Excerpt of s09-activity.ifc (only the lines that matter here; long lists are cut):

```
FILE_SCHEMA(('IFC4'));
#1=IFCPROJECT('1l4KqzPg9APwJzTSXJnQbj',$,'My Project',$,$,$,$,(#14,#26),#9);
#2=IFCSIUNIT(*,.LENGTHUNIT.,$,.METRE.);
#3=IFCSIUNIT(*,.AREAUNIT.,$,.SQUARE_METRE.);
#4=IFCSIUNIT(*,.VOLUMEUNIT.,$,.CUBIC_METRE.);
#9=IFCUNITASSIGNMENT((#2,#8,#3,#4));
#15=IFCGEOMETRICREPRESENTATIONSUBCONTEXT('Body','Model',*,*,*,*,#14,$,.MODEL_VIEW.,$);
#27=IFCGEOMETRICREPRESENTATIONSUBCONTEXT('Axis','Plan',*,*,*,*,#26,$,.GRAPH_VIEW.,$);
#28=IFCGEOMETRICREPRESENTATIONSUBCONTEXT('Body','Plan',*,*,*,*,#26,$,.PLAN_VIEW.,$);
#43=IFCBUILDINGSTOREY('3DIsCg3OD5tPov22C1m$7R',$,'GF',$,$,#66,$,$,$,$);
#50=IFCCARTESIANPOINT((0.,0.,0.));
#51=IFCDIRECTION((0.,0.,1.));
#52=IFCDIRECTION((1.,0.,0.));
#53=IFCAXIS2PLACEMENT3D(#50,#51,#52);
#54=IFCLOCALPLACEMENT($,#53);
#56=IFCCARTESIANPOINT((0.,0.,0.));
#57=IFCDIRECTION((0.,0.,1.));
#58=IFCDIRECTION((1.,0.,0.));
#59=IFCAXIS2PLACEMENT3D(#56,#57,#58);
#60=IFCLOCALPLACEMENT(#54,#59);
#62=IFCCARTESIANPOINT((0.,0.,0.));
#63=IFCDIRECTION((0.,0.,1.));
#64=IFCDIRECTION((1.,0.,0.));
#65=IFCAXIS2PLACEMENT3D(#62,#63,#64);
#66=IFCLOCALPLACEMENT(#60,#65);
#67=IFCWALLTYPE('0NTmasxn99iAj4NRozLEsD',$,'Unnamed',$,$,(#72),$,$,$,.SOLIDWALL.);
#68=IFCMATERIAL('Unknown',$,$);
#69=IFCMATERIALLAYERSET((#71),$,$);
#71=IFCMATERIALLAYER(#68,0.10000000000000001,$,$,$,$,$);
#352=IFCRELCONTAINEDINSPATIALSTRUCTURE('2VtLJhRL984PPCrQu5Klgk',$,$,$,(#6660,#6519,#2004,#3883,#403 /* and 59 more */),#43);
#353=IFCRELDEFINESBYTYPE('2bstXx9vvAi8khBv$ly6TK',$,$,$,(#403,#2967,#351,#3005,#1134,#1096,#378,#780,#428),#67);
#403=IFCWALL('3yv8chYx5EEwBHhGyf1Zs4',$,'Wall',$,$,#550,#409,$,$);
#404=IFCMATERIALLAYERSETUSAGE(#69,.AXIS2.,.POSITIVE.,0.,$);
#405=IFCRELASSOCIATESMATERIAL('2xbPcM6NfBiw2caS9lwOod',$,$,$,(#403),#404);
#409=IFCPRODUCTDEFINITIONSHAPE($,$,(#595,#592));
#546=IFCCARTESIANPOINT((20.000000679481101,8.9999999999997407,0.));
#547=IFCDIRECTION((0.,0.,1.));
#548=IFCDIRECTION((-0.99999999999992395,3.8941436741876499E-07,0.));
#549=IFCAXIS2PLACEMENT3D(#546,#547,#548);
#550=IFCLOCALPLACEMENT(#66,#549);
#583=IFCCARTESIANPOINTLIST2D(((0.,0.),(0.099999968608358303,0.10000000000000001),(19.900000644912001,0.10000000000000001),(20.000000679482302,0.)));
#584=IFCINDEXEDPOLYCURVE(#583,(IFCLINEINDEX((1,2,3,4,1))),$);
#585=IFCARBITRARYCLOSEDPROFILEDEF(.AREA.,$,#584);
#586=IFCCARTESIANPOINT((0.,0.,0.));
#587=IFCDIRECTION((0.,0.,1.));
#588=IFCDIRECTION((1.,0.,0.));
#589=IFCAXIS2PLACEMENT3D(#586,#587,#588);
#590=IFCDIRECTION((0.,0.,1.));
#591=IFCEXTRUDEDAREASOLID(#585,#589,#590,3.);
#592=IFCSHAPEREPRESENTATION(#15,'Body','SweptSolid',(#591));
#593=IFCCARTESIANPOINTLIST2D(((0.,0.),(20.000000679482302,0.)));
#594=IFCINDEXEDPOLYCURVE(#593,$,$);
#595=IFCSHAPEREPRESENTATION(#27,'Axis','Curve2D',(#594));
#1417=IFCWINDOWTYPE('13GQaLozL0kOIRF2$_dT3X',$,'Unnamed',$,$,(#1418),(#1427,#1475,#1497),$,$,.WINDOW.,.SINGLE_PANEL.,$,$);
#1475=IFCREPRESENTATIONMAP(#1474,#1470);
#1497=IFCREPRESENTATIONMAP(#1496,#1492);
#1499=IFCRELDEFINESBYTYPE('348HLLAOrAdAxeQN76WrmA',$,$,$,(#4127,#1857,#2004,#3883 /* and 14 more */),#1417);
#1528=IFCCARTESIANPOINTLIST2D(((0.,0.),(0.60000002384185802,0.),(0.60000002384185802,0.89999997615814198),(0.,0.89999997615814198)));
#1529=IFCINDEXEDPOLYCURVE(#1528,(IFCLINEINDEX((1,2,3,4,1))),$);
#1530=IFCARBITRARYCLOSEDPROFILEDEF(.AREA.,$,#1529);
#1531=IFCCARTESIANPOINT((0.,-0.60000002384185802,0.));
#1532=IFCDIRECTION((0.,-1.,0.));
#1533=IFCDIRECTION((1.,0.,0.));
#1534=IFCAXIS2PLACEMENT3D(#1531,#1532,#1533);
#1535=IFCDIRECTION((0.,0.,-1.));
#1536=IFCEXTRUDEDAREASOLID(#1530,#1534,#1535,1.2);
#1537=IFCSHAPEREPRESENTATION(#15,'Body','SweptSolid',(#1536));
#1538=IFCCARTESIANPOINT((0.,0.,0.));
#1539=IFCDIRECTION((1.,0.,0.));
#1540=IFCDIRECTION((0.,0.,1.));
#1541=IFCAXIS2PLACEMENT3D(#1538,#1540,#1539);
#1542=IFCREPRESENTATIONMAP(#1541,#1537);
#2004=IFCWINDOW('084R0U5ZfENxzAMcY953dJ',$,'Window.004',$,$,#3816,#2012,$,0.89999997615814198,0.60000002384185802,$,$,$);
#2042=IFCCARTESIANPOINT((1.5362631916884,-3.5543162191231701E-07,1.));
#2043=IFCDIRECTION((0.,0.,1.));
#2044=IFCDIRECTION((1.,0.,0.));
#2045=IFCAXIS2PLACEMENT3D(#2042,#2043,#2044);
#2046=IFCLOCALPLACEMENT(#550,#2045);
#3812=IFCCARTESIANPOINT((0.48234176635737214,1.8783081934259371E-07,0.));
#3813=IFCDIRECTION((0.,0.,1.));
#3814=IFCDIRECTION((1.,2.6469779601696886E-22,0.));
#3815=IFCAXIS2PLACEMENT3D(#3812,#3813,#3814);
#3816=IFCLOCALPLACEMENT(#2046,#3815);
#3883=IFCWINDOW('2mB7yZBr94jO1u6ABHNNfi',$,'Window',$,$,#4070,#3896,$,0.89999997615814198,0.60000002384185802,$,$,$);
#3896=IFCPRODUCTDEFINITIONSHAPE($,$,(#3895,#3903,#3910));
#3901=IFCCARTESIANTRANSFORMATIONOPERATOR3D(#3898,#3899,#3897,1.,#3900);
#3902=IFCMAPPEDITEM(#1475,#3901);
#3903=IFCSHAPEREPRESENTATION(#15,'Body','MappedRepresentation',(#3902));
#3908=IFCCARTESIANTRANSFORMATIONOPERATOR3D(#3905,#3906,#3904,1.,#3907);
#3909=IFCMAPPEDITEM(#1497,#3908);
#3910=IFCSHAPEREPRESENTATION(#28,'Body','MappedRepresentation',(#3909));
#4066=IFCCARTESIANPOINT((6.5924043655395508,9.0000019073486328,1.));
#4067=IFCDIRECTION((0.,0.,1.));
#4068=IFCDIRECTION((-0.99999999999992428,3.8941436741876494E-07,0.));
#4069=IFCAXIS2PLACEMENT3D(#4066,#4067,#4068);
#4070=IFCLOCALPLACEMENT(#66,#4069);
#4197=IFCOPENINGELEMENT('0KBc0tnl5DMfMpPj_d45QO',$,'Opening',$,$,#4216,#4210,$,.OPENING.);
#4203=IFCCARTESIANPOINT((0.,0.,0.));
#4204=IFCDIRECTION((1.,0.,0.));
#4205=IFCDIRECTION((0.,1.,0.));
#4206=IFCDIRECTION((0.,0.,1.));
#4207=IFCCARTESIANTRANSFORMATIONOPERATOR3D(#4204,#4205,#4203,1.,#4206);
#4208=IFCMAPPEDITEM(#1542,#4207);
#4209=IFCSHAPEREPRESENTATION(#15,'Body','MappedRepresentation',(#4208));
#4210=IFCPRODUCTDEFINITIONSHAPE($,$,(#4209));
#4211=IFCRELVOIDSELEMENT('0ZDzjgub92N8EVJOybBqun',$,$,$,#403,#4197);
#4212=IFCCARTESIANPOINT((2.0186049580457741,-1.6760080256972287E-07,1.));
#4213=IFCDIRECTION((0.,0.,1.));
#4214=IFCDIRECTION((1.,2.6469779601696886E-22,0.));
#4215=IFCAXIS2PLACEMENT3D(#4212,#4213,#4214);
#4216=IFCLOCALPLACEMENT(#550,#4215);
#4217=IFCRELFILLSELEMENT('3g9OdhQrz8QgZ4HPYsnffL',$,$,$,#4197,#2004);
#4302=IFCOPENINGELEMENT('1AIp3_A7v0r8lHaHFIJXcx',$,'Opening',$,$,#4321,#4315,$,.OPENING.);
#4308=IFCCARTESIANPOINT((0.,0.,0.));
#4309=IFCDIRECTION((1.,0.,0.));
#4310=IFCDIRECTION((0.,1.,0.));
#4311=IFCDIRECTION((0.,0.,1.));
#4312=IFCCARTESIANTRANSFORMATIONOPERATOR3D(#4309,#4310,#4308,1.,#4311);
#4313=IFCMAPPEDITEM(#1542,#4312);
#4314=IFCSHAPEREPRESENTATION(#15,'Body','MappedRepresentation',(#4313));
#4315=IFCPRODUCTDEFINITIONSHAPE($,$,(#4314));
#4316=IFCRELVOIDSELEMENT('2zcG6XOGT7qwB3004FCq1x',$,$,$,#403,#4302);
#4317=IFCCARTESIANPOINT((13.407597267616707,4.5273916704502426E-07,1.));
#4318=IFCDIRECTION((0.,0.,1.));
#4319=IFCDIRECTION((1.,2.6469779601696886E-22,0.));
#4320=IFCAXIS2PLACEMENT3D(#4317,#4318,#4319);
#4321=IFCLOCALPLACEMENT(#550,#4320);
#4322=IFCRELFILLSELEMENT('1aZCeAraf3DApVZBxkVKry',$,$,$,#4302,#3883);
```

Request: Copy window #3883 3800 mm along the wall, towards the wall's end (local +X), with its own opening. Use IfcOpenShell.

```python
import ifcopenshell
import ifcopenshell.api.feature
import ifcopenshell.api.geometry
import ifcopenshell.api.root
import ifcopenshell.geom
import ifcopenshell.util.element
import ifcopenshell.util.placement
import ifcopenshell.util.shape
import ifcopenshell.util.unit

model = ifcopenshell.open("s09-activity.ifc")
unit_scale = ifcopenshell.util.unit.calculate_unit_scale(model)
settings = ifcopenshell.geom.settings()


def volume(element):
    """Net volume in cubic metres, openings subtracted."""
    shape = ifcopenshell.geom.create_shape(settings, element)
    return ifcopenshell.util.shape.get_volume(shape.geometry)


window = model.by_guid("2mB7yZBr94jO1u6ABHNNfi")
opening = window.FillsVoids[0].RelatingOpeningElement
wall = opening.VoidsElements[0].RelatingBuildingElement
before = volume(wall)
shift = ifcopenshell.util.placement.get_local_placement(wall.ObjectPlacement)[:3, 0] * 3.8 / unit_scale

# copy_class copies the void relationship, type, container and properties, but no geometry.
new_opening = ifcopenshell.api.root.copy_class(model, product=opening)
new_opening.Representation = ifcopenshell.util.element.copy_deep(
    model, opening.Representation, exclude=["IfcGeometricRepresentationContext", "IfcRepresentationMap"]
)
new_window = ifcopenshell.api.root.copy_class(model, product=window)
new_window.Representation = ifcopenshell.util.element.copy_deep(
    model, window.Representation, exclude=["IfcGeometricRepresentationContext", "IfcRepresentationMap"]
)
ifcopenshell.api.feature.add_filling(model, opening=new_opening, element=new_window)

for old, new in ((opening, new_opening), (window, new_window)):
    matrix = ifcopenshell.util.placement.get_local_placement(old.ObjectPlacement)
    matrix[:3, 3] += shift
    ifcopenshell.api.geometry.edit_object_placement(model, product=new, matrix=matrix, is_si=False)

after = volume(wall)

print(f"wall volume {before:.3f} -> {after:.3f} m3")

model.write("s09-activity_rev.ifc")
```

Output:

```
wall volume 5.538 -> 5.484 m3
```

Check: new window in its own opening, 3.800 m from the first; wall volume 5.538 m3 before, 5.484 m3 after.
